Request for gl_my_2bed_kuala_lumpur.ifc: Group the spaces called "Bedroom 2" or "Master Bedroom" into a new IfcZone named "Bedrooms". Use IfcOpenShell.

First a look at what the model holds.

```python
import ifcopenshell

model = ifcopenshell.open("gl_my_2bed_kuala_lumpur.ifc")
print(model.schema)
seen = {}
for space in model.by_type("IfcSpace"):
    seen[space.LongName] = seen.get(space.LongName, 0) + 1
for name, count in sorted(seen.items(), key=str):
    print(count, "x", name)
print("zones:", [z.Name for z in model.by_type("IfcZone")][:20])
```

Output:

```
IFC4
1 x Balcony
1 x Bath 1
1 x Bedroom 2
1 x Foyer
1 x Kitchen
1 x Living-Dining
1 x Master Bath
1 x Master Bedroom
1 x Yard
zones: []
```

```python
import ifcopenshell
import ifcopenshell.api.group
import ifcopenshell.api.root

model = ifcopenshell.open("gl_my_2bed_kuala_lumpur.ifc")

names = {"Bedroom 2", "Master Bedroom"}
spaces = [s for s in model.by_type("IfcSpace") if s.LongName in names]

zone = ifcopenshell.api.root.create_entity(model, ifc_class="IfcZone", name="Bedrooms")
ifcopenshell.api.group.assign_group(model, products=spaces, group=zone)
print(len(spaces), "spaces in", zone.Name)

model.write("gl_my_2bed_kuala_lumpur_rev.ifc")
```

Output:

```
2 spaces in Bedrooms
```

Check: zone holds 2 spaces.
